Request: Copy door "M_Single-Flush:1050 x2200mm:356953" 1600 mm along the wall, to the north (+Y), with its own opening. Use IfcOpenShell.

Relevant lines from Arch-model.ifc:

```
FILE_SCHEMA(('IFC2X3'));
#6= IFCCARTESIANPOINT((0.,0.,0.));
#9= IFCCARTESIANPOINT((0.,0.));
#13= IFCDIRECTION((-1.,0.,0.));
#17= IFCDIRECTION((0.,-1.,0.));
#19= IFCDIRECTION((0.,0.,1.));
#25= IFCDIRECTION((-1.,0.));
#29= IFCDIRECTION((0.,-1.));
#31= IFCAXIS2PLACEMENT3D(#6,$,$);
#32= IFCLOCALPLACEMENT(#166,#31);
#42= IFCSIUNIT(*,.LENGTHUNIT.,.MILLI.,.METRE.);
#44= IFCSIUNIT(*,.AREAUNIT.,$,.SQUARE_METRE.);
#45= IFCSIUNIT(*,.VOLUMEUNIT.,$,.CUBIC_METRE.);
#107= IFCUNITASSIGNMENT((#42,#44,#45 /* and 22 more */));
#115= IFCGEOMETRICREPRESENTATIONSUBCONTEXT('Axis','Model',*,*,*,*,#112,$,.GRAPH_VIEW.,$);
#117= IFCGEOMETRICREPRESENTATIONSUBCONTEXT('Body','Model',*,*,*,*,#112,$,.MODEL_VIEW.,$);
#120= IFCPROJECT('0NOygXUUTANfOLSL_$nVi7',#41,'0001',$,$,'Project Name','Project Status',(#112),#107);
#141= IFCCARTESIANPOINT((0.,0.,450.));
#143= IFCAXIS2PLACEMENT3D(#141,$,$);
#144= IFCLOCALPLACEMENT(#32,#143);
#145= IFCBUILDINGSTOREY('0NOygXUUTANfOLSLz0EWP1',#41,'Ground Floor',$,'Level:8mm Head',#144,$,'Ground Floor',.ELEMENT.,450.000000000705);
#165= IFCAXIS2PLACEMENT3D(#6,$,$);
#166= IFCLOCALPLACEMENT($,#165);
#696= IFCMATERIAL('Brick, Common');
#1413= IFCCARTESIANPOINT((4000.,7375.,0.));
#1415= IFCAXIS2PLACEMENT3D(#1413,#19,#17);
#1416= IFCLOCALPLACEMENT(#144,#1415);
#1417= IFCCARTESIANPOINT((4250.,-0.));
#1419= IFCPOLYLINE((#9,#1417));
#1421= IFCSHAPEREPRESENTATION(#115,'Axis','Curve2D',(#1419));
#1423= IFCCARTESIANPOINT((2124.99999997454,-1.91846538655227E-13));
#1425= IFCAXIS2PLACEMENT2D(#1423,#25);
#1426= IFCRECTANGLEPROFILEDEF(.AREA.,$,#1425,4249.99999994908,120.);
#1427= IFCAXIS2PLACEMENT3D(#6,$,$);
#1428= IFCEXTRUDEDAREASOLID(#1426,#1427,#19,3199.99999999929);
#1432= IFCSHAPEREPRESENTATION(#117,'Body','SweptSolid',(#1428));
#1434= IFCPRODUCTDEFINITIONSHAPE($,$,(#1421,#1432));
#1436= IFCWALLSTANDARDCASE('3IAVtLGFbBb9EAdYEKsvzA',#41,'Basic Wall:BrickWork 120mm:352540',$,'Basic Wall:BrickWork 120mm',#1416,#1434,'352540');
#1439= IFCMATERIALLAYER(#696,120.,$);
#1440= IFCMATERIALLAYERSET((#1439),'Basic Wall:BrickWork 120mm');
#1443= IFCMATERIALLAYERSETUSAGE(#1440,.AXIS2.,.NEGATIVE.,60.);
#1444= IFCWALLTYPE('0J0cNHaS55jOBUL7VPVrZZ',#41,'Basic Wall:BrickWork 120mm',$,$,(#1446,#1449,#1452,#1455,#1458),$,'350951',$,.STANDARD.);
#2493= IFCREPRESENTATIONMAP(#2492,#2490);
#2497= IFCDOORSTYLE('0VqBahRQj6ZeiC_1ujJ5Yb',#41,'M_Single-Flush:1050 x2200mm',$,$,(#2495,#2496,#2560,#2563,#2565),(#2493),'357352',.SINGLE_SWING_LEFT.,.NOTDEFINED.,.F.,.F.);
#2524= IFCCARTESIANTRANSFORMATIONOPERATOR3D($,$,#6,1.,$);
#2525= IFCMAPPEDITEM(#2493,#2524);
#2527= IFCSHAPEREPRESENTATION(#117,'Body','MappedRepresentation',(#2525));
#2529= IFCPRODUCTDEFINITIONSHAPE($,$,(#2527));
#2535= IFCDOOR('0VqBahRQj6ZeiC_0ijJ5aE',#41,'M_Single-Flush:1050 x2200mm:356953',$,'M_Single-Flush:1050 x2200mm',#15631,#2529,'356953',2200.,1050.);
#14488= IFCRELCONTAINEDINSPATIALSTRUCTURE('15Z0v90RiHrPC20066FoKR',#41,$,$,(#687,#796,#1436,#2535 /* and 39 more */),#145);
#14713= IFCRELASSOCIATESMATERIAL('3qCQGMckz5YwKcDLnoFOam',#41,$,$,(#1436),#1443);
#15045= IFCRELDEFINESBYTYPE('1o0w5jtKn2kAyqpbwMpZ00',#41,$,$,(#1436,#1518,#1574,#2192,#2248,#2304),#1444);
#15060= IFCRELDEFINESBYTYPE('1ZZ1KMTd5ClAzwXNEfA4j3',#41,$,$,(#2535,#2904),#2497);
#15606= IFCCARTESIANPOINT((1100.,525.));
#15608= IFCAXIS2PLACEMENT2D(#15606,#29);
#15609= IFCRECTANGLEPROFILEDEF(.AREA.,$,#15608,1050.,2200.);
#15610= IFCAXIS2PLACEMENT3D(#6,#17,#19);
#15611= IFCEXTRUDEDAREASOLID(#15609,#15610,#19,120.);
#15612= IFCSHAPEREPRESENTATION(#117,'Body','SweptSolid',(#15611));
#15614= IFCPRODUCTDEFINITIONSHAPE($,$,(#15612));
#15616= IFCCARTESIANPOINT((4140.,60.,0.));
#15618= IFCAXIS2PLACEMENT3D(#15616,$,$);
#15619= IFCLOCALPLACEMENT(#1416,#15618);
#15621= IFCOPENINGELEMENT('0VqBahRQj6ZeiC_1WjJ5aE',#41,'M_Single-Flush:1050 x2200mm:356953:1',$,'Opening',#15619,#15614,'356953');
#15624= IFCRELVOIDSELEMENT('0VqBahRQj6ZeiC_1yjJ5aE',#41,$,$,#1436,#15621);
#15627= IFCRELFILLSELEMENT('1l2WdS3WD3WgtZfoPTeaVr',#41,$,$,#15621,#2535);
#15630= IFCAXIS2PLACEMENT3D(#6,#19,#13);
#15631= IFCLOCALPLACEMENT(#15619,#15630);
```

```python
import ifcopenshell
import ifcopenshell.api.feature
import ifcopenshell.api.geometry
import ifcopenshell.api.root
import ifcopenshell.geom
import ifcopenshell.util.element
import ifcopenshell.util.placement
import ifcopenshell.util.shape
import ifcopenshell.util.unit

model = ifcopenshell.open("Arch-model.ifc")
unit_scale = ifcopenshell.util.unit.calculate_unit_scale(model)
settings = ifcopenshell.geom.settings()


def volume(element):
    """Net volume in cubic metres, openings subtracted."""
    shape = ifcopenshell.geom.create_shape(settings, element)
    return ifcopenshell.util.shape.get_volume(shape.geometry)


def reuse_history(source, copy):
    """copy_class also copies each property set's owner history, people and application; keep the originals."""
    for rel in copy.IsDefinedBy:
        if rel.is_a("IfcRelDefinesByProperties") and (history := rel.RelatingPropertyDefinition.OwnerHistory):
            rel.RelatingPropertyDefinition.OwnerHistory = source.OwnerHistory
            ifcopenshell.util.element.remove_deep2(model, history)


door = model.by_guid("0VqBahRQj6ZeiC_0ijJ5aE")
opening = door.FillsVoids[0].RelatingOpeningElement
wall = opening.VoidsElements[0].RelatingBuildingElement
before = volume(wall)
shift = ifcopenshell.util.placement.get_local_placement(wall.ObjectPlacement)[:3, 0] * -1.6 / unit_scale

# copy_class copies the void relationship, type, container and properties, but no geometry.
new_opening = ifcopenshell.api.root.copy_class(model, product=opening)
new_opening.Representation = ifcopenshell.util.element.copy_deep(
    model, opening.Representation, exclude=["IfcGeometricRepresentationContext", "IfcRepresentationMap"]
)
new_opening.Name = "M_Single-Flush:1050 x2200mm"
new_opening.Tag = None
new_door = ifcopenshell.api.root.copy_class(model, product=door)
new_door.Representation = ifcopenshell.util.element.copy_deep(
    model, door.Representation, exclude=["IfcGeometricRepresentationContext", "IfcRepresentationMap"]
)
new_door.Name = "M_Single-Flush:1050 x2200mm"
new_door.Tag = None
reuse_history(door, new_door)
fills = ifcopenshell.api.feature.add_filling(model, opening=new_opening, element=new_door)
fills.OwnerHistory = new_door.OwnerHistory  # required in IFC2X3

for old, new in ((opening, new_opening), (door, new_door)):
    matrix = ifcopenshell.util.placement.get_local_placement(old.ObjectPlacement)
    matrix[:3, 3] += shift
    ifcopenshell.api.geometry.edit_object_placement(model, product=new, matrix=matrix, is_si=False)

after = volume(wall)

print(f"wall volume {before:.3f} -> {after:.3f} m3")

model.write("Arch-model_v2.ifc")
```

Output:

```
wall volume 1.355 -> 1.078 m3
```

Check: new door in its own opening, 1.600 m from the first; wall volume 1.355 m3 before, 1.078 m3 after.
